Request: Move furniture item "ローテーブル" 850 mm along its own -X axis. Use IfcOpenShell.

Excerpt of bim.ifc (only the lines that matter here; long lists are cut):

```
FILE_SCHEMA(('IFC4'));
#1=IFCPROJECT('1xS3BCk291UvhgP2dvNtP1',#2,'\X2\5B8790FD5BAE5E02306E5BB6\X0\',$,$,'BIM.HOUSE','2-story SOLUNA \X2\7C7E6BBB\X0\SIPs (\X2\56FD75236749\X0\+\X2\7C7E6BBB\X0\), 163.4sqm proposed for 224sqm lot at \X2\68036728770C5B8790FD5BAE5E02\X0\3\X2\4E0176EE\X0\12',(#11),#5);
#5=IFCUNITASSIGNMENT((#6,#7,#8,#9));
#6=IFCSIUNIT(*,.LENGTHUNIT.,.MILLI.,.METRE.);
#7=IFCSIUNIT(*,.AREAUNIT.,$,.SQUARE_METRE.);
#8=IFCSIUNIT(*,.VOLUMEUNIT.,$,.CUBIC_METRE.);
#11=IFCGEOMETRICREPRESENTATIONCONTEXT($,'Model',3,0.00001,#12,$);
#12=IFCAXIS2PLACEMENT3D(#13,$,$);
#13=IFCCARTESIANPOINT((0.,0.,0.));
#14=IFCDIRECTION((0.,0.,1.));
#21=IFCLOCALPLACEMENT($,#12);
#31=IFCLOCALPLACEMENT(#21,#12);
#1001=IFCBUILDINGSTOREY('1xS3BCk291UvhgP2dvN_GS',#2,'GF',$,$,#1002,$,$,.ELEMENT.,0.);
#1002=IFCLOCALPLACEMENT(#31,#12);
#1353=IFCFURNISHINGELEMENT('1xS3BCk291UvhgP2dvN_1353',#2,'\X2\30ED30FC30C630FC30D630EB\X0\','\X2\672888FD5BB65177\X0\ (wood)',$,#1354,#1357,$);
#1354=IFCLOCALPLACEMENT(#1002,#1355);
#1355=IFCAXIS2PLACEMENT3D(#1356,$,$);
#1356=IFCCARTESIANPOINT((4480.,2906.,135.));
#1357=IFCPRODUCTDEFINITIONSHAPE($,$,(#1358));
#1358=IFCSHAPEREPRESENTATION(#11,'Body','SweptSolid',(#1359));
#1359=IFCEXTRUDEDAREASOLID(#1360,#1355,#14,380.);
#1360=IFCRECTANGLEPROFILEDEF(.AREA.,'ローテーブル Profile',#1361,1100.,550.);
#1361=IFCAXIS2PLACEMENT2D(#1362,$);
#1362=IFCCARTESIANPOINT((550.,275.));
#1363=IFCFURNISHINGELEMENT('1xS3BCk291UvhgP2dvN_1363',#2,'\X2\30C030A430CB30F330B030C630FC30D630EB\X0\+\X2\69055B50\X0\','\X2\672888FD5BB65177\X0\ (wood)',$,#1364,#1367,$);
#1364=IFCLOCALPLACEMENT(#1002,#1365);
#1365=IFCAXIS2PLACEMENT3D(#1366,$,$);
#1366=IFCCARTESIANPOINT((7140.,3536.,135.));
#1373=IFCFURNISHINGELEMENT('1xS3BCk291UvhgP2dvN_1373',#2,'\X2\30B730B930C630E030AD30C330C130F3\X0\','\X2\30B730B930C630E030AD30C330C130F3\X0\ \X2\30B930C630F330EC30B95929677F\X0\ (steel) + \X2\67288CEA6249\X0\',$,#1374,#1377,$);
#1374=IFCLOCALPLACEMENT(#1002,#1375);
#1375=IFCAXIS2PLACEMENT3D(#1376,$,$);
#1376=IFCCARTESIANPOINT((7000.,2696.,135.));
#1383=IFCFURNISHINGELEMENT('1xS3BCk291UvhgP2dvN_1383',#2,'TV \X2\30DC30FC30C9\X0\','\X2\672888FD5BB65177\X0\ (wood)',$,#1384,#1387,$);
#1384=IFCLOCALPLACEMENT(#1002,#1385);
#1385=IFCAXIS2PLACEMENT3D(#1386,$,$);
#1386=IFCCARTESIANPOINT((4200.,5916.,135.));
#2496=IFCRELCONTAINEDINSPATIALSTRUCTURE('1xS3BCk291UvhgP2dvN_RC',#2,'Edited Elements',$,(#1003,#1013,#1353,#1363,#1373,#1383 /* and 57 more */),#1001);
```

```python
import ifcopenshell
import ifcopenshell.api.geometry
import ifcopenshell.util.placement
import ifcopenshell.util.unit

model = ifcopenshell.open("bim.ifc")
unit_scale = ifcopenshell.util.unit.calculate_unit_scale(model)

item = model.by_guid("1xS3BCk291UvhgP2dvN_1353")
matrix = ifcopenshell.util.placement.get_local_placement(item.ObjectPlacement)
matrix[:3, 3] -= matrix[:3, 0] * 0.85 / unit_scale
ifcopenshell.api.geometry.edit_object_placement(model, product=item, matrix=matrix, is_si=False)

print(ifcopenshell.util.placement.get_local_placement(item.ObjectPlacement).round(3) + 0.0)

model.write("bim-out.ifc")
```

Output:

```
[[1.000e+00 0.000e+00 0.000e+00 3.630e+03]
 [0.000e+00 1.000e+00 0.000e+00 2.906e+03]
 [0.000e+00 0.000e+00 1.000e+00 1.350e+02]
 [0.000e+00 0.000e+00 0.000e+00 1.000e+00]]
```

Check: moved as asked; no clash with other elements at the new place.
